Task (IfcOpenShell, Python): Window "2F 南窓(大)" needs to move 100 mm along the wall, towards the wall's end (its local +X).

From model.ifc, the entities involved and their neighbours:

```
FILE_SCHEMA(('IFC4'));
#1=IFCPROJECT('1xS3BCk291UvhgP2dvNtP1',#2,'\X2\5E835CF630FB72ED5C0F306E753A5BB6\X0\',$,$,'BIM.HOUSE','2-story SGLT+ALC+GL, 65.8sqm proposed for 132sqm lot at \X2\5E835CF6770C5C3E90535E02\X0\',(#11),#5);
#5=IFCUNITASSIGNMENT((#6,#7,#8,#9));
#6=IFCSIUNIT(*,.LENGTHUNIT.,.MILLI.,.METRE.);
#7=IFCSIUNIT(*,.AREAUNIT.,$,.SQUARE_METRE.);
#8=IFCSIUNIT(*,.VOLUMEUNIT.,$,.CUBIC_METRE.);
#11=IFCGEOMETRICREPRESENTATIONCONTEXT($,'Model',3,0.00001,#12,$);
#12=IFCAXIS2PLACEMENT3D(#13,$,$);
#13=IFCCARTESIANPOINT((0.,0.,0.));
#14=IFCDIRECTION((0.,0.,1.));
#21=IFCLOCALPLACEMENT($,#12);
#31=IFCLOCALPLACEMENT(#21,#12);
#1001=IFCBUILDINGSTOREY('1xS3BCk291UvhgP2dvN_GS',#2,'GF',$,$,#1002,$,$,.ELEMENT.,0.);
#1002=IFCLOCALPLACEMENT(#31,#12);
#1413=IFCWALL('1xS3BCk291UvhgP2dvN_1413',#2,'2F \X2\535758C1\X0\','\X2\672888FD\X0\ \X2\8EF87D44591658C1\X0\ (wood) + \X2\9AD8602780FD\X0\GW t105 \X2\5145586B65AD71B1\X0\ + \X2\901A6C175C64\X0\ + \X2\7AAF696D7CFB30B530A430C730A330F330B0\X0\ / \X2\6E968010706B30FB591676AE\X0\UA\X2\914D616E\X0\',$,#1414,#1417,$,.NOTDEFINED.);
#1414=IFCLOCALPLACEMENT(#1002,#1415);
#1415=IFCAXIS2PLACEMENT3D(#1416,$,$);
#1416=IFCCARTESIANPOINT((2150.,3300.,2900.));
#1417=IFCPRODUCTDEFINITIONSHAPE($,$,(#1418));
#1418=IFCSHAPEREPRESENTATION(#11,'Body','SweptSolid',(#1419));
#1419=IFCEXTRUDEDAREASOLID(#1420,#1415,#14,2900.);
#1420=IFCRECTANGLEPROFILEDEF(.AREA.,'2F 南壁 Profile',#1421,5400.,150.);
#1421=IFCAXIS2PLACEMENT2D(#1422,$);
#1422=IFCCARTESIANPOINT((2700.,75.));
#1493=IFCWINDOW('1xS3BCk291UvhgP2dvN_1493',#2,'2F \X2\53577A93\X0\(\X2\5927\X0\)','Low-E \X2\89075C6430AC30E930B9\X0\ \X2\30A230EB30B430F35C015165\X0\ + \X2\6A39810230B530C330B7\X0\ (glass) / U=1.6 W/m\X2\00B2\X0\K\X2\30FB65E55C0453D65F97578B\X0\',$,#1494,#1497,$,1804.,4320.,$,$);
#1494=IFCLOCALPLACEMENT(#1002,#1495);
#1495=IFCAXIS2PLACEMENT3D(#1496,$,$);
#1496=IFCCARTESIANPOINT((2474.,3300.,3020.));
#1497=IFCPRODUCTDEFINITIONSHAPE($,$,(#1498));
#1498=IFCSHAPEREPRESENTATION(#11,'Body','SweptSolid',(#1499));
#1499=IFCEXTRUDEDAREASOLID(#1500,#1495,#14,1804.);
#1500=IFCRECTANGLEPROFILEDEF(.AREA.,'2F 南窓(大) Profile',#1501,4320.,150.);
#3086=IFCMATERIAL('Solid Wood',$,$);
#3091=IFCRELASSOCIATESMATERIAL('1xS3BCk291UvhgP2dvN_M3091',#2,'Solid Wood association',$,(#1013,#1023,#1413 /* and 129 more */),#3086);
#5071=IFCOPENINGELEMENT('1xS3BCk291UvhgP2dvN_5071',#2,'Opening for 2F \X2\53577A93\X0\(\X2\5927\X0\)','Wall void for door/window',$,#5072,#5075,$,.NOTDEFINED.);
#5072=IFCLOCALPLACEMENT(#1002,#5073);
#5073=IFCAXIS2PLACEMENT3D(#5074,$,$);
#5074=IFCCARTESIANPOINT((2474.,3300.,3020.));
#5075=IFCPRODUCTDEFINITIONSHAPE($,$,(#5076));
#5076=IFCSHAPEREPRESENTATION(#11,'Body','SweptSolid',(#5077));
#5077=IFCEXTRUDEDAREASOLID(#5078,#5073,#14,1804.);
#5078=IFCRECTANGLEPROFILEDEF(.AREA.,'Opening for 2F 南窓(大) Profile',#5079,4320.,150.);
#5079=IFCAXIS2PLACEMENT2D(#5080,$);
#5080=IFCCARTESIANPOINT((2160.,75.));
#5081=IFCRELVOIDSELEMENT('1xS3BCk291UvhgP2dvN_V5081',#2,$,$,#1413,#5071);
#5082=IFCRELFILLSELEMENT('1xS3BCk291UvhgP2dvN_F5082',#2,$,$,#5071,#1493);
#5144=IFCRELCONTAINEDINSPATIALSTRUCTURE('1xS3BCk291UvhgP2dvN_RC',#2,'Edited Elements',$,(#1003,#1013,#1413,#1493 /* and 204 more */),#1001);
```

```python
import ifcopenshell
import ifcopenshell.api.geometry
import ifcopenshell.util.placement

model = ifcopenshell.open("model.ifc")

window = model.by_id(1493)
opening = window.FillsVoids[0].RelatingOpeningElement
wall = opening.VoidsElements[0].RelatingBuildingElement

wall_matrix = ifcopenshell.util.placement.get_local_placement(wall.ObjectPlacement)
shift = wall_matrix[:3, 0] * 100.0
before = ifcopenshell.util.placement.get_local_placement(window.ObjectPlacement)[:3, 3].copy()

# The window is not placed relative to its opening, so move both.
for product in (opening, window):
    matrix = ifcopenshell.util.placement.get_local_placement(product.ObjectPlacement)
    matrix[:3, 3] += shift
    ifcopenshell.api.geometry.edit_object_placement(model, product=product, matrix=matrix, is_si=False)

after = ifcopenshell.util.placement.get_local_placement(window.ObjectPlacement)[:3, 3]
print("window moved by", (after - before).round(3) + 0.0)

model.write("model_edited.ifc")
```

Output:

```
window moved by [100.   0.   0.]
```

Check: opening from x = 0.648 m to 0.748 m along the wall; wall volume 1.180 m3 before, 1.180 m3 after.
